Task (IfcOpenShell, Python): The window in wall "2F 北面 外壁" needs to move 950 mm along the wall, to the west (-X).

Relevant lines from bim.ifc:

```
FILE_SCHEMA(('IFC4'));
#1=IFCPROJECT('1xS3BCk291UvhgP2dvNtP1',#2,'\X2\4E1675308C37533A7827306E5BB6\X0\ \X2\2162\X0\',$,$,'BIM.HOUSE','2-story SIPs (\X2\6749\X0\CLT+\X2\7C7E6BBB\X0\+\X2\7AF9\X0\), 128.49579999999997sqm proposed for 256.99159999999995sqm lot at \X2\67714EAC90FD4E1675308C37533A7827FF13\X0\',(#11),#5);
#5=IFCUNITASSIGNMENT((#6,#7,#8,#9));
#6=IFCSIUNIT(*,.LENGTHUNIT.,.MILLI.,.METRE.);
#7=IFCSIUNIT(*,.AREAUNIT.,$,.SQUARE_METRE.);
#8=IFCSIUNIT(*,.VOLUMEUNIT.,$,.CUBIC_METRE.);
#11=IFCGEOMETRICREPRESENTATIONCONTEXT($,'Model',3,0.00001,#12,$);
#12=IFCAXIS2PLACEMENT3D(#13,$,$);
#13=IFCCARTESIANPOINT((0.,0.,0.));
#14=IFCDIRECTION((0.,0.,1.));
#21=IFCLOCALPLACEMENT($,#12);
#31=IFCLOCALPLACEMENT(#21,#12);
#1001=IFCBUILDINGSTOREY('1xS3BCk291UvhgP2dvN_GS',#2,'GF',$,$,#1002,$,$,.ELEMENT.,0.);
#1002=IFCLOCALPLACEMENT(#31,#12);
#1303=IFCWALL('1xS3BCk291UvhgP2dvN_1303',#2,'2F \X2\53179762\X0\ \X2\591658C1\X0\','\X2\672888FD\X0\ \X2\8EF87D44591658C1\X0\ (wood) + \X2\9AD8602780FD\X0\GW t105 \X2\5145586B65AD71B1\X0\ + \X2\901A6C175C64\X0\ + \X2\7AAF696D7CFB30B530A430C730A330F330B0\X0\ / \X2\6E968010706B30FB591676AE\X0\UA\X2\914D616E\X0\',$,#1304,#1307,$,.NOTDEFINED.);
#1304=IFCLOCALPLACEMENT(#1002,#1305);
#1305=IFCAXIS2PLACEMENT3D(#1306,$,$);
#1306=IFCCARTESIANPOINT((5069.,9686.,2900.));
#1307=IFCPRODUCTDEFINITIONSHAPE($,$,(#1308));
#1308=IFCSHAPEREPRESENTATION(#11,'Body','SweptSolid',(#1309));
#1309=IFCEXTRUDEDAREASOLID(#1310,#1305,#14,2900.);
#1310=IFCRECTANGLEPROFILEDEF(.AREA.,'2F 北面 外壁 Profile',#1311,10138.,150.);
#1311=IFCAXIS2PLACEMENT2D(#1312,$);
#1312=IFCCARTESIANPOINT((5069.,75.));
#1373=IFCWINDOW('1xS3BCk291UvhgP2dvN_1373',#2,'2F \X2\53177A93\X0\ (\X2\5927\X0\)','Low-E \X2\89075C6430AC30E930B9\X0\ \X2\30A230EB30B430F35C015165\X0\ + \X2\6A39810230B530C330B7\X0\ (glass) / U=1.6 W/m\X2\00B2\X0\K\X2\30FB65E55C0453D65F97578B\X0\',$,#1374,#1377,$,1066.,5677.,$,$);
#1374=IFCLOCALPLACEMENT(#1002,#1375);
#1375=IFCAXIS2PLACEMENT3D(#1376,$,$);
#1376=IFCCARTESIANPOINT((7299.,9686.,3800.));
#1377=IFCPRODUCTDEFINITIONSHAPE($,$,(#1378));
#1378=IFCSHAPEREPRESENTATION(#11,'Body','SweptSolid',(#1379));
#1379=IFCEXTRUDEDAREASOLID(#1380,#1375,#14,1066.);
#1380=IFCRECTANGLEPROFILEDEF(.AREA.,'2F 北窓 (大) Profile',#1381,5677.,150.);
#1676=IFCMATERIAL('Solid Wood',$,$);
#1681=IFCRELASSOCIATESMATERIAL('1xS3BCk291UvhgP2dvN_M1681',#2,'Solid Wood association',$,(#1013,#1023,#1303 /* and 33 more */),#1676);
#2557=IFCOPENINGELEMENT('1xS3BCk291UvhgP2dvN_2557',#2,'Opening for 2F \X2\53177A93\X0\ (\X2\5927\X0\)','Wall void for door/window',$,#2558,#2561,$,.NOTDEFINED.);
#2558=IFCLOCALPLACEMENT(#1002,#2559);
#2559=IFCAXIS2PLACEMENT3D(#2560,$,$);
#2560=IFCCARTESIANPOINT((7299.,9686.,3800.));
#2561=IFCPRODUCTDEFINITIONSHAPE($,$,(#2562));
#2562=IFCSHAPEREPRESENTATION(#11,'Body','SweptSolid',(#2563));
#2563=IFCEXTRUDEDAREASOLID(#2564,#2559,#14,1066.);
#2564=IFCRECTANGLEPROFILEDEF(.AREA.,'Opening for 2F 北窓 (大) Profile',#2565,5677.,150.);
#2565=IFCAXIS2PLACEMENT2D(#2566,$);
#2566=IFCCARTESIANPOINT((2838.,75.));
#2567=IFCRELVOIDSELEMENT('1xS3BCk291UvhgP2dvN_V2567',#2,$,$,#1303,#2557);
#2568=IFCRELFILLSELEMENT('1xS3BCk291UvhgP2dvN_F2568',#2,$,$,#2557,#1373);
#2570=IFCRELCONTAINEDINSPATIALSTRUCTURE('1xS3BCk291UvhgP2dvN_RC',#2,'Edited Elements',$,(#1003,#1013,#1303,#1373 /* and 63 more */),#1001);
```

```python
import ifcopenshell
import ifcopenshell.api.geometry
import ifcopenshell.util.placement
import ifcopenshell.util.unit

model = ifcopenshell.open("bim.ifc")
unit_scale = ifcopenshell.util.unit.calculate_unit_scale(model)

window = model.by_id(1373)
opening = window.FillsVoids[0].RelatingOpeningElement
wall = opening.VoidsElements[0].RelatingBuildingElement

wall_matrix = ifcopenshell.util.placement.get_local_placement(wall.ObjectPlacement)
shift = wall_matrix[:3, 0] * -0.95 / unit_scale
before = ifcopenshell.util.placement.get_local_placement(window.ObjectPlacement)[:3, 3].copy()

# The window is not placed relative to its opening, so move both.
for product in (opening, window):
    matrix = ifcopenshell.util.placement.get_local_placement(product.ObjectPlacement)
    matrix[:3, 3] += shift
    ifcopenshell.api.geometry.edit_object_placement(model, product=product, matrix=matrix, is_si=False)

after = ifcopenshell.util.placement.get_local_placement(window.ObjectPlacement)[:3, 3]
print("window moved by", (after - before).round(3) + 0.0)

model.write("bim_rev.ifc")
```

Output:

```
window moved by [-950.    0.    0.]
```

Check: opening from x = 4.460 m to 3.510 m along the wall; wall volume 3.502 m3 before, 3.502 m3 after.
